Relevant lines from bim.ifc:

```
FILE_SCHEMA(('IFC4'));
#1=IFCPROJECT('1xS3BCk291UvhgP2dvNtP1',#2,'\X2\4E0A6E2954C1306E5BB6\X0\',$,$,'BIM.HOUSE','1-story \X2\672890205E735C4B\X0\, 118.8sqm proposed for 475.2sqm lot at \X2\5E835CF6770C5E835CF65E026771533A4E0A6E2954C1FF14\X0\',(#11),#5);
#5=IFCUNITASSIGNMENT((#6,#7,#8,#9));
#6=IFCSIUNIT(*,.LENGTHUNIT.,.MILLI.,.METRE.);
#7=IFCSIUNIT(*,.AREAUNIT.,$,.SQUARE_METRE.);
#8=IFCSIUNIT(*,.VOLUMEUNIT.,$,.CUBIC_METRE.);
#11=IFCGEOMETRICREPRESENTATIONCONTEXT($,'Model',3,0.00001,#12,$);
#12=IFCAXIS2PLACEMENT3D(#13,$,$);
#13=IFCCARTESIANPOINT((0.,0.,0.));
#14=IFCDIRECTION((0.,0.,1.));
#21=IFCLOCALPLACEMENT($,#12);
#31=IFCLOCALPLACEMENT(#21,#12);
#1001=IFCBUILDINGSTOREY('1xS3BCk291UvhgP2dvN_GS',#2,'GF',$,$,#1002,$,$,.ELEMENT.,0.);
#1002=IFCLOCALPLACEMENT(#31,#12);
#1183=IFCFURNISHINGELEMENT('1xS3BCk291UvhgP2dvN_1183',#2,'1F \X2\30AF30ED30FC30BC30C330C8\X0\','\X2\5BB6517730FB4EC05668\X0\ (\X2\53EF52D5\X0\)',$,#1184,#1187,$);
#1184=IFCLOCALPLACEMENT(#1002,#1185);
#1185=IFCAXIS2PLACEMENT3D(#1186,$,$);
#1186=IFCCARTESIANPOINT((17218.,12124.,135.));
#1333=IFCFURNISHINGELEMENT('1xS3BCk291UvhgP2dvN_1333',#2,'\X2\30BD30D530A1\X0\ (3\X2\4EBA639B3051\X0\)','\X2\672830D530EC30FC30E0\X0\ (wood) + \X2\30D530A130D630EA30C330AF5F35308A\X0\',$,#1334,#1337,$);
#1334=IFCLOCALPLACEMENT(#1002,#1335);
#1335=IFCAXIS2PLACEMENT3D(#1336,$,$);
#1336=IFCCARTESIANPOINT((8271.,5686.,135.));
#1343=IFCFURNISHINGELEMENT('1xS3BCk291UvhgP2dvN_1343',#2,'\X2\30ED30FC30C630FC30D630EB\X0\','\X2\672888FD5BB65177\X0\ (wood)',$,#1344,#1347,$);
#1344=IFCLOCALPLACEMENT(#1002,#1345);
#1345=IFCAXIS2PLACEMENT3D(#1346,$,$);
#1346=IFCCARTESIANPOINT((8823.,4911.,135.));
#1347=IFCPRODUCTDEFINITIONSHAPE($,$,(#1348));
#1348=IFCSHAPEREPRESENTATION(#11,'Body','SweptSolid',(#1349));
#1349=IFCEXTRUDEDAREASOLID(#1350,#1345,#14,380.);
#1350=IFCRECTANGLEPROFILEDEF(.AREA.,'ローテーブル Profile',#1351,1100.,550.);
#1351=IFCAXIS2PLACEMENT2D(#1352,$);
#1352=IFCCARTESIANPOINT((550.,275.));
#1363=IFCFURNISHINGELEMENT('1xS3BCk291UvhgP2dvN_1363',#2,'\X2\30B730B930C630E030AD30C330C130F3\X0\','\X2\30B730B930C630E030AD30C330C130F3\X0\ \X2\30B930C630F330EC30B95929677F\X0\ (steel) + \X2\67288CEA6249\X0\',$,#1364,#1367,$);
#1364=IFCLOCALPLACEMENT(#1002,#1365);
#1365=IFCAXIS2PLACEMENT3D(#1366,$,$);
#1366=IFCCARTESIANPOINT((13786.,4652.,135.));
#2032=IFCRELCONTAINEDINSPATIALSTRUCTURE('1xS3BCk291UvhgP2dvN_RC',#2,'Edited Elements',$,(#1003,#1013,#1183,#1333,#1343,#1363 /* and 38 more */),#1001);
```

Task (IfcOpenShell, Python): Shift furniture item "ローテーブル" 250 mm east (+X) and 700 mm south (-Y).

```python
import ifcopenshell
import ifcopenshell.api.geometry
import ifcopenshell.util.placement
import ifcopenshell.util.unit

model = ifcopenshell.open("bim.ifc")
unit_scale = ifcopenshell.util.unit.calculate_unit_scale(model)

item = model.by_guid("1xS3BCk291UvhgP2dvN_1343")
matrix = ifcopenshell.util.placement.get_local_placement(item.ObjectPlacement)
matrix[0, 3] += 0.25 / unit_scale
matrix[1, 3] -= 0.7 / unit_scale
ifcopenshell.api.geometry.edit_object_placement(model, product=item, matrix=matrix, is_si=False)

print(ifcopenshell.util.placement.get_local_placement(item.ObjectPlacement).round(3) + 0.0)

model.write("bim_edited.ifc")
```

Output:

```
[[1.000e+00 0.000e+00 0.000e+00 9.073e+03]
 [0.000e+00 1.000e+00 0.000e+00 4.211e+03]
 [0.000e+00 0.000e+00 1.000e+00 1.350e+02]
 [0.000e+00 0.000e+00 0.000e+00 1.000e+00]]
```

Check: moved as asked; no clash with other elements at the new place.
